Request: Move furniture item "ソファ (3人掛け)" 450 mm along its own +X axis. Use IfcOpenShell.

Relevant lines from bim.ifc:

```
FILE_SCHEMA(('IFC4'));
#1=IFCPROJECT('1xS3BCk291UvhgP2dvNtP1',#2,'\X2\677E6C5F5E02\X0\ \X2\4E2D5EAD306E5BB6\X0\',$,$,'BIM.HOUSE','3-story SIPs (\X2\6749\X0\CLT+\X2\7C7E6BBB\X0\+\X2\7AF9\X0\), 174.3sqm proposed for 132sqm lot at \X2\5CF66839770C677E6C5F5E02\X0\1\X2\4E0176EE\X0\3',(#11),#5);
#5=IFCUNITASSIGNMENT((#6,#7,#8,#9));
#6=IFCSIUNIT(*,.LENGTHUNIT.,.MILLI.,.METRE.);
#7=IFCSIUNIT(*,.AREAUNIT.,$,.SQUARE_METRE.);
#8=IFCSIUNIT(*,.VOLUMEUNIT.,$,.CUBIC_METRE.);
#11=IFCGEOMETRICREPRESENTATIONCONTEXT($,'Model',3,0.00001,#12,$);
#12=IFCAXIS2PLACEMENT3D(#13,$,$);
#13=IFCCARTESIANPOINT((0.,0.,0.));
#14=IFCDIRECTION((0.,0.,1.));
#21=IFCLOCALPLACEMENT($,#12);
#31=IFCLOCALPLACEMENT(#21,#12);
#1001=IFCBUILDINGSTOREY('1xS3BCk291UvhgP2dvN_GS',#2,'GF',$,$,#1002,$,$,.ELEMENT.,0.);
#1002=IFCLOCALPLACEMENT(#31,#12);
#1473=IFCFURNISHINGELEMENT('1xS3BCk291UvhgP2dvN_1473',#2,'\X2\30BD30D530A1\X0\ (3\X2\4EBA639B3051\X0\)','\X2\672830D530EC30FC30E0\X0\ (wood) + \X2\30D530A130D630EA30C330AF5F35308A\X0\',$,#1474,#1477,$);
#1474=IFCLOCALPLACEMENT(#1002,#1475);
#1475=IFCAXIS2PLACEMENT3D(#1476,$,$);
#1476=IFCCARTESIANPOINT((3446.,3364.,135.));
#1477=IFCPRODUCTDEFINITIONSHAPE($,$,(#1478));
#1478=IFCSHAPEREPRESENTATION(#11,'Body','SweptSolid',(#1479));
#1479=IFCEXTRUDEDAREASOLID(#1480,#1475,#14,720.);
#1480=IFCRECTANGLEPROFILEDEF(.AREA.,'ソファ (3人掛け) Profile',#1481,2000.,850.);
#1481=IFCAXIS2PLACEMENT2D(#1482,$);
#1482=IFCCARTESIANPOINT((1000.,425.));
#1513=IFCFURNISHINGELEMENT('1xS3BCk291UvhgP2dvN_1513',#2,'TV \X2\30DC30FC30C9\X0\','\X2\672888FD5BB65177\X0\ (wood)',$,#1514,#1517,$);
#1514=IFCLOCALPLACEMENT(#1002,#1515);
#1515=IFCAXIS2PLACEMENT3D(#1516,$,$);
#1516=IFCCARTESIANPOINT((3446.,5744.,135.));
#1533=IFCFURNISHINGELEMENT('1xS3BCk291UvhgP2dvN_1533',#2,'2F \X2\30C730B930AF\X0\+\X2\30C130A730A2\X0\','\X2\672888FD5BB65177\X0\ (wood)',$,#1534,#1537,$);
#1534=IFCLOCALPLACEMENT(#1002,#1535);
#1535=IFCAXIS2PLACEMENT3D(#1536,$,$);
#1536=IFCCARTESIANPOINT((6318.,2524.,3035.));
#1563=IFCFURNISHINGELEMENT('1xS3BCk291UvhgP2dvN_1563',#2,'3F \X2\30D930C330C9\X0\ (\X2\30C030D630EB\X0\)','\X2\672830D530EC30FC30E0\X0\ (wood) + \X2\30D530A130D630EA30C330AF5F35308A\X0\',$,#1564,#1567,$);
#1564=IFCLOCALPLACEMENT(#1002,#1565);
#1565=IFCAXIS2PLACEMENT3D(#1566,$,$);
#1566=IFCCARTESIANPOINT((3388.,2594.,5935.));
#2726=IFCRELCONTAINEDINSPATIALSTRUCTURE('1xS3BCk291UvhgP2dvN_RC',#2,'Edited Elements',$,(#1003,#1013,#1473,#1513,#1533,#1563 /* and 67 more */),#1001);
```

```python
import ifcopenshell
import ifcopenshell.api.geometry
import ifcopenshell.util.placement

model = ifcopenshell.open("bim.ifc")

item = model.by_id(1473)
matrix = ifcopenshell.util.placement.get_local_placement(item.ObjectPlacement)
matrix[:3, 3] += matrix[:3, 0] * 450.0
ifcopenshell.api.geometry.edit_object_placement(model, product=item, matrix=matrix, is_si=False)

print(ifcopenshell.util.placement.get_local_placement(item.ObjectPlacement).round(3) + 0.0)

model.write("bim_edited.ifc")
```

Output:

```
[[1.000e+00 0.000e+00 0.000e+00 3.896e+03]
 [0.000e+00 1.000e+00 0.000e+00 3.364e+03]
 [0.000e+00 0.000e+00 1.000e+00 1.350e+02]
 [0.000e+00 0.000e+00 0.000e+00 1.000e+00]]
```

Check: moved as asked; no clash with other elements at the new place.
